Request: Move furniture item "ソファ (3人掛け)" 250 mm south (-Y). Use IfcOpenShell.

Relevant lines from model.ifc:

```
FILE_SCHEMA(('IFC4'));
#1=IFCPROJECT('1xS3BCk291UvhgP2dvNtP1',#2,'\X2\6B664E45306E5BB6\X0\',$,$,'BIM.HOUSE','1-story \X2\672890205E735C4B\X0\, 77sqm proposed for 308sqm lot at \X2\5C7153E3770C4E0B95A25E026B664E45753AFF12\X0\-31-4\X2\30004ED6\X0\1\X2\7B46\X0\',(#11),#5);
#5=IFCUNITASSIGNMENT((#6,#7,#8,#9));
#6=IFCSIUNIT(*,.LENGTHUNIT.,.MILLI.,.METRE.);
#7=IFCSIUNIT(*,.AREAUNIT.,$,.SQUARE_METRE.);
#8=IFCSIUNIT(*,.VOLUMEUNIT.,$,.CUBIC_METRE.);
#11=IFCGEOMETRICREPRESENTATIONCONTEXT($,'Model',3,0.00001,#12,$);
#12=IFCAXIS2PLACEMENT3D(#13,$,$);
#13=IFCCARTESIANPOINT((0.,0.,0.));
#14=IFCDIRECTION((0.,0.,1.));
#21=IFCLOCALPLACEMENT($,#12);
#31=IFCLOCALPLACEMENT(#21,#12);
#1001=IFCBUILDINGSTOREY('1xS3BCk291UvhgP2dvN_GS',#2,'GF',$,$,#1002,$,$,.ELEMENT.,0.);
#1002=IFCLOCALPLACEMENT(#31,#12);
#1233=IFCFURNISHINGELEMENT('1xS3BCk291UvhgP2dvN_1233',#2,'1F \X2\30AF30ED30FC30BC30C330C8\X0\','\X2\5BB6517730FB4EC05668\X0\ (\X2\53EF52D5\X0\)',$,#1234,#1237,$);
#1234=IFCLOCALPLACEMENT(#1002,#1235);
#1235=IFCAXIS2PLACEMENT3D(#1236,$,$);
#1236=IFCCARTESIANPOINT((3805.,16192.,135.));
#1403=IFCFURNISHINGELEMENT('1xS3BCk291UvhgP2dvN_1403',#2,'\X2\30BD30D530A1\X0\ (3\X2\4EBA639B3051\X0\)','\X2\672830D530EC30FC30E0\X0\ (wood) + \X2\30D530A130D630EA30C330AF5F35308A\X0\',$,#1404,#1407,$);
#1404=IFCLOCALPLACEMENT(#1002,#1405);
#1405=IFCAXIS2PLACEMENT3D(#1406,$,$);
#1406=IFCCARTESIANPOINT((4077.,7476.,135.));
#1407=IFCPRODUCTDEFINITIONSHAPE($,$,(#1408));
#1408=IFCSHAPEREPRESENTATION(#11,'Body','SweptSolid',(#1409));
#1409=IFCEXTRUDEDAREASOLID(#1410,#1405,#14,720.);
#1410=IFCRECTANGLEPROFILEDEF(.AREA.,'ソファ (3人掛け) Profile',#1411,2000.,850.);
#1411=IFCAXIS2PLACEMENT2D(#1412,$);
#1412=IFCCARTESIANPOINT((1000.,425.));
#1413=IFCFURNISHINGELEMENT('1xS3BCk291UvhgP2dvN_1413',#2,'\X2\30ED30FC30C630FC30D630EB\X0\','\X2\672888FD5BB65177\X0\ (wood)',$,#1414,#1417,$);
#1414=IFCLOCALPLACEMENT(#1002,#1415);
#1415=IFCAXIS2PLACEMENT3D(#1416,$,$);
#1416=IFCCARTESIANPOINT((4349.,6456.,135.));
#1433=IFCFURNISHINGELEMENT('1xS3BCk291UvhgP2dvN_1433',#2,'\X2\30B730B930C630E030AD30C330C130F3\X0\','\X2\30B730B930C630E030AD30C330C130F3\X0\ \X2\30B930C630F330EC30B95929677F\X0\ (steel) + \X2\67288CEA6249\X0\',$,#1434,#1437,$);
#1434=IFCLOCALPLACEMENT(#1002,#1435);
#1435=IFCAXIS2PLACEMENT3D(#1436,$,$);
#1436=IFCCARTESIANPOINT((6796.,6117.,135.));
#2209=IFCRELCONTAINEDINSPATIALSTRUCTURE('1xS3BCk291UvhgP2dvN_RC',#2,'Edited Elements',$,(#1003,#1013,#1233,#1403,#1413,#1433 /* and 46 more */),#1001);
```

```python
import ifcopenshell
import ifcopenshell.api.geometry
import ifcopenshell.util.placement
import ifcopenshell.util.unit

model = ifcopenshell.open("model.ifc")
unit_scale = ifcopenshell.util.unit.calculate_unit_scale(model)

item = model.by_id(1403)
matrix = ifcopenshell.util.placement.get_local_placement(item.ObjectPlacement)
matrix[1, 3] -= 0.25 / unit_scale
ifcopenshell.api.geometry.edit_object_placement(model, product=item, matrix=matrix, is_si=False)

print(ifcopenshell.util.placement.get_local_placement(item.ObjectPlacement).round(3) + 0.0)

model.write("model_updated.ifc")
```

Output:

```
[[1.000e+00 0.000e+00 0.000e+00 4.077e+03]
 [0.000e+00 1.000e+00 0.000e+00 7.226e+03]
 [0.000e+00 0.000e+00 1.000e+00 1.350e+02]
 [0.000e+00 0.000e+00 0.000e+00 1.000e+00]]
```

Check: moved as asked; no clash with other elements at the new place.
